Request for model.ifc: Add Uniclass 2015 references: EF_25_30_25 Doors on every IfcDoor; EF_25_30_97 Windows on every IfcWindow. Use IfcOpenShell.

First a look at what the model holds.

```python
import ifcopenshell

model = ifcopenshell.open("model.ifc")
print(model.schema)
print("classifications:", [c.Name for c in model.by_type("IfcClassification")])
for ifc_class in ("IfcDoor", "IfcRoof", "IfcStair", "IfcWall", "IfcWindow"):
    print(ifc_class, len(model.by_type(ifc_class)))
```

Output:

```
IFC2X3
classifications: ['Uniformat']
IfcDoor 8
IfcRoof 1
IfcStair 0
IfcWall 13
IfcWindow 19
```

```python
import ifcopenshell
import ifcopenshell.api.classification

model = ifcopenshell.open("model.ifc")

# IFC2X3 requires Source and Edition and has no link from the project to the system.
system = model.create_entity("IfcClassification", Source="NBS", Edition="2015", Name="Uniclass 2015")

codes = {
    "IfcDoor": ("EF_25_30_25", "Doors"),
    "IfcWindow": ("EF_25_30_97", "Windows"),
}
for ifc_class, (code, name) in codes.items():
    products = model.by_type(ifc_class)
    ifcopenshell.api.classification.add_reference(
        model, products=products, classification=system, identification=code, name=name
    )
    print(code, len(products))

model.write("model_updated.ifc")
```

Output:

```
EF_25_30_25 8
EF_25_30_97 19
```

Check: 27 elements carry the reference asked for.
